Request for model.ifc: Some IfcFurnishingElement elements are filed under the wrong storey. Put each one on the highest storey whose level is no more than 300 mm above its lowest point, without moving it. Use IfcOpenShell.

First a look at what the model holds.

```python
import ifcopenshell
import ifcopenshell.util.element
import ifcopenshell.util.placement

model = ifcopenshell.open("model.ifc")
print(model.schema)
for storey in model.by_type("IfcBuildingStorey"):
    level = ifcopenshell.util.placement.get_storey_elevation(storey)
    count = sum(e.is_a("IfcFurnishingElement") for e in ifcopenshell.util.element.get_contained(storey))
    print(storey.id(), storey.Name, round(level, 3), count, sep=" | ")
```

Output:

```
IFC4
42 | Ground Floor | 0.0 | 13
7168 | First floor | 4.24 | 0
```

```python
import ifcopenshell
import ifcopenshell.api.spatial
import ifcopenshell.geom
import ifcopenshell.util.element
import ifcopenshell.util.placement
import ifcopenshell.util.shape
import ifcopenshell.util.unit

model = ifcopenshell.open("model.ifc")
unit_scale = ifcopenshell.util.unit.calculate_unit_scale(model)
settings = ifcopenshell.geom.settings()

levels = sorted(
    ((ifcopenshell.util.placement.get_storey_elevation(s) * unit_scale, s) for s in model.by_type("IfcBuildingStorey")),
    key=lambda pair: pair[0],
)

for e in model.by_type("IfcFurnishingElement"):
    current = e.ContainedInStructure[0].RelatingStructure if e.ContainedInStructure else None
    if current is None or not current.is_a("IfcBuildingStorey"):
        continue
    shape = ifcopenshell.geom.create_shape(settings, e)
    bottom = ifcopenshell.util.shape.get_shape_bottom_elevation(shape, shape.geometry)
    below = [s for level, s in levels if level <= bottom + 0.3]
    storey = below[-1] if below else levels[0][1]
    if storey != current:
        # assign_container keeps the world position.
        ifcopenshell.api.spatial.assign_container(model, products=[e], relating_structure=storey)
        print(e.id(), current.Name, "->", storey.Name)

model.write("model_edited.ifc")
```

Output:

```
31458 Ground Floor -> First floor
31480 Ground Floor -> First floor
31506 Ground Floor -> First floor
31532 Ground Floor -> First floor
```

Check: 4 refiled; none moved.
